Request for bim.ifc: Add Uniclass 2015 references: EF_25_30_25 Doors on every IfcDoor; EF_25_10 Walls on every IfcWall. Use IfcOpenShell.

First a look at what the model holds.

```python
import ifcopenshell

model = ifcopenshell.open("bim.ifc")
print(model.schema)
print("classifications:", [c.Name for c in model.by_type("IfcClassification")])
for ifc_class in ("IfcDoor", "IfcRoof", "IfcStair", "IfcWall", "IfcWindow"):
    print(ifc_class, len(model.by_type(ifc_class)))
```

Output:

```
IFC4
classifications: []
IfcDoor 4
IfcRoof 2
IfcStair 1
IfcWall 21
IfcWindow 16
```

```python
import ifcopenshell
import ifcopenshell.api.classification

model = ifcopenshell.open("bim.ifc")

system = ifcopenshell.api.classification.add_classification(model, classification="Uniclass 2015")

codes = {
    "IfcDoor": ("EF_25_30_25", "Doors"),
    "IfcWall": ("EF_25_10", "Walls"),
}
for ifc_class, (code, name) in codes.items():
    products = model.by_type(ifc_class)
    ifcopenshell.api.classification.add_reference(
        model, products=products, classification=system, identification=code, name=name
    )
    print(code, len(products))

model.write("bim_edited.ifc")
```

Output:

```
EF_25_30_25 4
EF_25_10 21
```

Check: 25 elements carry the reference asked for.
